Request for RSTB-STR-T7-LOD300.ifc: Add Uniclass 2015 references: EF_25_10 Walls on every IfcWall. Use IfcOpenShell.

First a look at what the model holds.

```python
import ifcopenshell

model = ifcopenshell.open("RSTB-STR-T7-LOD300.ifc")
print(model.schema)
print("classifications:", [c.Name for c in model.by_type("IfcClassification")])
for ifc_class in ("IfcDoor", "IfcRoof", "IfcStair", "IfcWall", "IfcWindow"):
    print(ifc_class, len(model.by_type(ifc_class)))
```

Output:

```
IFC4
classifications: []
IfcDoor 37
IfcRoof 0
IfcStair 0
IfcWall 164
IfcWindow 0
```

```python
import ifcopenshell
import ifcopenshell.api.classification

model = ifcopenshell.open("RSTB-STR-T7-LOD300.ifc")

system = ifcopenshell.api.classification.add_classification(model, classification="Uniclass 2015")

codes = {
    "IfcWall": ("EF_25_10", "Walls"),
}
for ifc_class, (code, name) in codes.items():
    products = model.by_type(ifc_class)
    ifcopenshell.api.classification.add_reference(
        model, products=products, classification=system, identification=code, name=name
    )
    print(code, len(products))

model.write("RSTB-STR-T7-LOD300_rev.ifc")
```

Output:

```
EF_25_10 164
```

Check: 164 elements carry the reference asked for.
